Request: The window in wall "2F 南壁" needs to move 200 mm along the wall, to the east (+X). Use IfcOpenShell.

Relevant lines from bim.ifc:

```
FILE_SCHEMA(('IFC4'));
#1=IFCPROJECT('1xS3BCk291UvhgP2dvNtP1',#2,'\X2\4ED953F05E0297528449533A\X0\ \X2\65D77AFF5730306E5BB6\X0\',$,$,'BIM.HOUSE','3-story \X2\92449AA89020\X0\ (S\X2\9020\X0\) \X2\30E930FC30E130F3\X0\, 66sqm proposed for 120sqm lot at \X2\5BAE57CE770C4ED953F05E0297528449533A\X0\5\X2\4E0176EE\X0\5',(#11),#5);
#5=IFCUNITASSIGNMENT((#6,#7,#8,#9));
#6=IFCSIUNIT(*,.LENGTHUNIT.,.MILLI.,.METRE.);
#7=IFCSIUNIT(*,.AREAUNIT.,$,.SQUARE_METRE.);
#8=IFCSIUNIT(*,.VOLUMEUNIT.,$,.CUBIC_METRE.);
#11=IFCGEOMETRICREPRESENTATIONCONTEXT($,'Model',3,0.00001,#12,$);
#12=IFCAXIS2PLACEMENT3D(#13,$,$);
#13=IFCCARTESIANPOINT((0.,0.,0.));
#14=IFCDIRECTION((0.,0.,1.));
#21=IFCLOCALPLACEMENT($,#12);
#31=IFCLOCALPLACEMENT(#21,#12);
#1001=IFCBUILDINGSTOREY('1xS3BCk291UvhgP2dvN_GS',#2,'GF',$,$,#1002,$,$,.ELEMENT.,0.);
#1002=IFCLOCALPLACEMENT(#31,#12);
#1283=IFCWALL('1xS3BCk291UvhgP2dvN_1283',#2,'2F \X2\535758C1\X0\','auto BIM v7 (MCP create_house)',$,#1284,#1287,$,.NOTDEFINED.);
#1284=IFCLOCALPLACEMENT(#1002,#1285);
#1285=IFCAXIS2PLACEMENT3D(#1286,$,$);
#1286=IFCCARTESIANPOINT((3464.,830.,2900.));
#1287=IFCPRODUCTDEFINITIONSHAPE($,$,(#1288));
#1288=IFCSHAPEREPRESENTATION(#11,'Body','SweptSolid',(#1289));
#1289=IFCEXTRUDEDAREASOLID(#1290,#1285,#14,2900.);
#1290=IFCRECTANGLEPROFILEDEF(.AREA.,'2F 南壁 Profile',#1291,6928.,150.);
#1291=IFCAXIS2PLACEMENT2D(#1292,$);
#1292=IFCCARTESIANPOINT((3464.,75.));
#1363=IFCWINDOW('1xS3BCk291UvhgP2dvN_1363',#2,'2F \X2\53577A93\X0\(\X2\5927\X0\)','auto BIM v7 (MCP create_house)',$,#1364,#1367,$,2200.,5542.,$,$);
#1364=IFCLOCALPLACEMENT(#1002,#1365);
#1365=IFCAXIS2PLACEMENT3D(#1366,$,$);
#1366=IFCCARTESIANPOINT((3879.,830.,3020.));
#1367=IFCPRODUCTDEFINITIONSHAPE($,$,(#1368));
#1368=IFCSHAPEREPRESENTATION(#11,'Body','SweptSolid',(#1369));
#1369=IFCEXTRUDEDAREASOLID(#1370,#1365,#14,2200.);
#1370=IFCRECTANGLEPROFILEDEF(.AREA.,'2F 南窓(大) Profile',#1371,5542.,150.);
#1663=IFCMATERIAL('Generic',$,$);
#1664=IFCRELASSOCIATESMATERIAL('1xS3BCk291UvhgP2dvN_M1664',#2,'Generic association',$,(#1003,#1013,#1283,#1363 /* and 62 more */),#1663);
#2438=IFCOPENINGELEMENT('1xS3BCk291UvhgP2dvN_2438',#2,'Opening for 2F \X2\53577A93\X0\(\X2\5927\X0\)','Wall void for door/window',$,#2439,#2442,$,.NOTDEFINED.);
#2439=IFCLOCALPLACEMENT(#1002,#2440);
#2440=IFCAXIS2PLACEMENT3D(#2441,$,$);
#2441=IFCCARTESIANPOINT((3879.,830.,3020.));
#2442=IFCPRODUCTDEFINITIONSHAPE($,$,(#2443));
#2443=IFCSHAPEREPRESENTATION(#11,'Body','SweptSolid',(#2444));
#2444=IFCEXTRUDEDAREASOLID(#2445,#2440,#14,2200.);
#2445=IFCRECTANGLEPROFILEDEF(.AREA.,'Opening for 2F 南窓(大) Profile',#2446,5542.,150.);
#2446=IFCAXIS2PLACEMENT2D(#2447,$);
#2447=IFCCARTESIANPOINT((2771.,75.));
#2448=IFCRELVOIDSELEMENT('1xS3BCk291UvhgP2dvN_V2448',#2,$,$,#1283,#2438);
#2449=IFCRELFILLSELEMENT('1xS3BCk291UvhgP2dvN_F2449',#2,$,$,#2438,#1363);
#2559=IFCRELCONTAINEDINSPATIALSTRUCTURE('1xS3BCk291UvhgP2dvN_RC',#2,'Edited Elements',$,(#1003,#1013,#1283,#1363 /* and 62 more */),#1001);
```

```python
import ifcopenshell
import ifcopenshell.api.geometry
import ifcopenshell.util.placement
import ifcopenshell.util.unit

model = ifcopenshell.open("bim.ifc")
unit_scale = ifcopenshell.util.unit.calculate_unit_scale(model)

window = model.by_guid("1xS3BCk291UvhgP2dvN_1363")
opening = window.FillsVoids[0].RelatingOpeningElement
wall = opening.VoidsElements[0].RelatingBuildingElement

wall_matrix = ifcopenshell.util.placement.get_local_placement(wall.ObjectPlacement)
shift = wall_matrix[:3, 0] * 0.2 / unit_scale
before = ifcopenshell.util.placement.get_local_placement(window.ObjectPlacement)[:3, 3].copy()

# The window is not placed relative to its opening, so move both.
for product in (opening, window):
    matrix = ifcopenshell.util.placement.get_local_placement(product.ObjectPlacement)
    matrix[:3, 3] += shift
    ifcopenshell.api.geometry.edit_object_placement(model, product=product, matrix=matrix, is_si=False)

after = ifcopenshell.util.placement.get_local_placement(window.ObjectPlacement)[:3, 3]
print("window moved by", (after - before).round(3) + 0.0)

model.write("bim_v2.ifc")
```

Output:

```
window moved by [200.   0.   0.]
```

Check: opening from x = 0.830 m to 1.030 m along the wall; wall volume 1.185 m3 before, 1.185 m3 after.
